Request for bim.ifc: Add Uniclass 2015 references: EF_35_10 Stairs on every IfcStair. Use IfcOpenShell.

First a look at what the model holds.

```python
import ifcopenshell

model = ifcopenshell.open("bim.ifc")
print(model.schema)
print("classifications:", [c.Name for c in model.by_type("IfcClassification")])
for ifc_class in ("IfcDoor", "IfcRoof", "IfcStair", "IfcWall", "IfcWindow"):
    print(ifc_class, len(model.by_type(ifc_class)))
```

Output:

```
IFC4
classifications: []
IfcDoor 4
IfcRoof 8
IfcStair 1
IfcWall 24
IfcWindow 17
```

```python
import ifcopenshell
import ifcopenshell.api.classification

model = ifcopenshell.open("bim.ifc")

system = ifcopenshell.api.classification.add_classification(model, classification="Uniclass 2015")

codes = {
    "IfcStair": ("EF_35_10", "Stairs"),
}
for ifc_class, (code, name) in codes.items():
    products = model.by_type(ifc_class)
    ifcopenshell.api.classification.add_reference(
        model, products=products, classification=system, identification=code, name=name
    )
    print(code, len(products))

model.write("bim_updated.ifc")
```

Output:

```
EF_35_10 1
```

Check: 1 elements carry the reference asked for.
